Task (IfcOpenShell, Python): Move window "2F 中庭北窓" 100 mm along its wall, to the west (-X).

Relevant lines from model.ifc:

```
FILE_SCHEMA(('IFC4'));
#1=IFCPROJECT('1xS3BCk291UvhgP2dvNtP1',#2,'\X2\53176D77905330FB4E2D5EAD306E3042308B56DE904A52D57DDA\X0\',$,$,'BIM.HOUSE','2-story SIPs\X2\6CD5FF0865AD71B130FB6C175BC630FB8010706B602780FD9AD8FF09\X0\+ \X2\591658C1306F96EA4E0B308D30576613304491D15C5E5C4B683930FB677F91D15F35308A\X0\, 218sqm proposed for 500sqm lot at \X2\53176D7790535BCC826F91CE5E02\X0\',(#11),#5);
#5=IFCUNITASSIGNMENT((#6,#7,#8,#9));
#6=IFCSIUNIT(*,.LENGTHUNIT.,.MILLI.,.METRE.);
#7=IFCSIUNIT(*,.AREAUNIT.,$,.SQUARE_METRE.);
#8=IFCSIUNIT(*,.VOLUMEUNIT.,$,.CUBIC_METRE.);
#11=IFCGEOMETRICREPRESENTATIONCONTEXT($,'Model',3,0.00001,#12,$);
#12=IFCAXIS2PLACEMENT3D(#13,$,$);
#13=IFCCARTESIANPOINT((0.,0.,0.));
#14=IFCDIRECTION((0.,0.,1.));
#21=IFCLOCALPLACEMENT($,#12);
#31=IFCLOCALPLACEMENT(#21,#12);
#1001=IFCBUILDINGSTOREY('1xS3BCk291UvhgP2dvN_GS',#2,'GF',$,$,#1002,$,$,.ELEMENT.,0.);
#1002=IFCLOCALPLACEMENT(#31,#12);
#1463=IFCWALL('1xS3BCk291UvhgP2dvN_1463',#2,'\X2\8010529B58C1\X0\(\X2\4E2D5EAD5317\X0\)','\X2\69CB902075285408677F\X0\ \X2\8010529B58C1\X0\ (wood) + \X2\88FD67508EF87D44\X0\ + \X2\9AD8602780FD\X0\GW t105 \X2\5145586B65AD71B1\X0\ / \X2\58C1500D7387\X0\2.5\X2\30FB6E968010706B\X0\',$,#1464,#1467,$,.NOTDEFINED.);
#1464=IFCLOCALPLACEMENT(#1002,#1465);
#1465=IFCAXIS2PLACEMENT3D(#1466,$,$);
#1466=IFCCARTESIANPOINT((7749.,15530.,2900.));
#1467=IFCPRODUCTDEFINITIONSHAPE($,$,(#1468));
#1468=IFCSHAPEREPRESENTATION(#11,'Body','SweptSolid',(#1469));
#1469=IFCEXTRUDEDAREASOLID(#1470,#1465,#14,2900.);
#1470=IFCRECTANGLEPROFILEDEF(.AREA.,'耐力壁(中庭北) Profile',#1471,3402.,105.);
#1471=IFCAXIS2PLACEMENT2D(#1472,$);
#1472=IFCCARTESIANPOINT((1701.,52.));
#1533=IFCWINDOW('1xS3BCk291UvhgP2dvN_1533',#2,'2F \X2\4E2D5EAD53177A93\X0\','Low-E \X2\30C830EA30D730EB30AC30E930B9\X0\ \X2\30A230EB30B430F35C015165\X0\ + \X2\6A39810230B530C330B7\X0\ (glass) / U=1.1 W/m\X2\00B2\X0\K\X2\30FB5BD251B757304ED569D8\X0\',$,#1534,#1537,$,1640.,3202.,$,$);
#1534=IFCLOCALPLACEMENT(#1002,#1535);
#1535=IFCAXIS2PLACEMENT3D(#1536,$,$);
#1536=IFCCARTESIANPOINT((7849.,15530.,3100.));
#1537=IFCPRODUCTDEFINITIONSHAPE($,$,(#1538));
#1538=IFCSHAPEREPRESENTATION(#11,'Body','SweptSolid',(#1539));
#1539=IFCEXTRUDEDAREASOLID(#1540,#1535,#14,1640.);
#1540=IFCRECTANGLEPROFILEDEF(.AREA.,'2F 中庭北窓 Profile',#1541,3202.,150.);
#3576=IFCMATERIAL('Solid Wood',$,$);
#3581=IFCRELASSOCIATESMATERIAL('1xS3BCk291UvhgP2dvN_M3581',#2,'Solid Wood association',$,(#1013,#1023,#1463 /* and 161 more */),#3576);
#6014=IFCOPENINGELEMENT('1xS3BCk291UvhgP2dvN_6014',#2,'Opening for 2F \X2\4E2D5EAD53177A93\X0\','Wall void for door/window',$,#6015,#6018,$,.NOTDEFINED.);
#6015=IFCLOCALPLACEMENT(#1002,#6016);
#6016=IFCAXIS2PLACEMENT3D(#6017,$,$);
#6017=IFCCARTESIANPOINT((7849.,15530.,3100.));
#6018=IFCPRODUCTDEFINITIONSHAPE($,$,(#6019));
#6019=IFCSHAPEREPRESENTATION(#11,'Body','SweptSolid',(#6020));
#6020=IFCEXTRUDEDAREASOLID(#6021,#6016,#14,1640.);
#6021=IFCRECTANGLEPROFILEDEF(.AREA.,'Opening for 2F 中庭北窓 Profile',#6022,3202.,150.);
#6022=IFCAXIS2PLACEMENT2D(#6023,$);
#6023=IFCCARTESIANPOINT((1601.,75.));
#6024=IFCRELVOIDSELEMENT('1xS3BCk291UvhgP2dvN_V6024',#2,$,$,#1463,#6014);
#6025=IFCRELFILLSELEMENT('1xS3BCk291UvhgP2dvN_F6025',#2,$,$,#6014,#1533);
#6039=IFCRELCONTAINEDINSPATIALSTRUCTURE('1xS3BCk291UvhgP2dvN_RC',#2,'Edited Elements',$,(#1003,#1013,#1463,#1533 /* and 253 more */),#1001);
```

```python
import ifcopenshell
import ifcopenshell.api.geometry
import ifcopenshell.util.placement

model = ifcopenshell.open("model.ifc")

window = model.by_id(1533)
opening = window.FillsVoids[0].RelatingOpeningElement
wall = opening.VoidsElements[0].RelatingBuildingElement

wall_matrix = ifcopenshell.util.placement.get_local_placement(wall.ObjectPlacement)
shift = wall_matrix[:3, 0] * -100.0
before = ifcopenshell.util.placement.get_local_placement(window.ObjectPlacement)[:3, 3].copy()

# The window is not placed relative to its opening, so move both.
for product in (opening, window):
    matrix = ifcopenshell.util.placement.get_local_placement(product.ObjectPlacement)
    matrix[:3, 3] += shift
    ifcopenshell.api.geometry.edit_object_placement(model, product=product, matrix=matrix, is_si=False)

after = ifcopenshell.util.placement.get_local_placement(window.ObjectPlacement)[:3, 3]
print("window moved by", (after - before).round(3) + 0.0)

model.write("model_updated.ifc")
```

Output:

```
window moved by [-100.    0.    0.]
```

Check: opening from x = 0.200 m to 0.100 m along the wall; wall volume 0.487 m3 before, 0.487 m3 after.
